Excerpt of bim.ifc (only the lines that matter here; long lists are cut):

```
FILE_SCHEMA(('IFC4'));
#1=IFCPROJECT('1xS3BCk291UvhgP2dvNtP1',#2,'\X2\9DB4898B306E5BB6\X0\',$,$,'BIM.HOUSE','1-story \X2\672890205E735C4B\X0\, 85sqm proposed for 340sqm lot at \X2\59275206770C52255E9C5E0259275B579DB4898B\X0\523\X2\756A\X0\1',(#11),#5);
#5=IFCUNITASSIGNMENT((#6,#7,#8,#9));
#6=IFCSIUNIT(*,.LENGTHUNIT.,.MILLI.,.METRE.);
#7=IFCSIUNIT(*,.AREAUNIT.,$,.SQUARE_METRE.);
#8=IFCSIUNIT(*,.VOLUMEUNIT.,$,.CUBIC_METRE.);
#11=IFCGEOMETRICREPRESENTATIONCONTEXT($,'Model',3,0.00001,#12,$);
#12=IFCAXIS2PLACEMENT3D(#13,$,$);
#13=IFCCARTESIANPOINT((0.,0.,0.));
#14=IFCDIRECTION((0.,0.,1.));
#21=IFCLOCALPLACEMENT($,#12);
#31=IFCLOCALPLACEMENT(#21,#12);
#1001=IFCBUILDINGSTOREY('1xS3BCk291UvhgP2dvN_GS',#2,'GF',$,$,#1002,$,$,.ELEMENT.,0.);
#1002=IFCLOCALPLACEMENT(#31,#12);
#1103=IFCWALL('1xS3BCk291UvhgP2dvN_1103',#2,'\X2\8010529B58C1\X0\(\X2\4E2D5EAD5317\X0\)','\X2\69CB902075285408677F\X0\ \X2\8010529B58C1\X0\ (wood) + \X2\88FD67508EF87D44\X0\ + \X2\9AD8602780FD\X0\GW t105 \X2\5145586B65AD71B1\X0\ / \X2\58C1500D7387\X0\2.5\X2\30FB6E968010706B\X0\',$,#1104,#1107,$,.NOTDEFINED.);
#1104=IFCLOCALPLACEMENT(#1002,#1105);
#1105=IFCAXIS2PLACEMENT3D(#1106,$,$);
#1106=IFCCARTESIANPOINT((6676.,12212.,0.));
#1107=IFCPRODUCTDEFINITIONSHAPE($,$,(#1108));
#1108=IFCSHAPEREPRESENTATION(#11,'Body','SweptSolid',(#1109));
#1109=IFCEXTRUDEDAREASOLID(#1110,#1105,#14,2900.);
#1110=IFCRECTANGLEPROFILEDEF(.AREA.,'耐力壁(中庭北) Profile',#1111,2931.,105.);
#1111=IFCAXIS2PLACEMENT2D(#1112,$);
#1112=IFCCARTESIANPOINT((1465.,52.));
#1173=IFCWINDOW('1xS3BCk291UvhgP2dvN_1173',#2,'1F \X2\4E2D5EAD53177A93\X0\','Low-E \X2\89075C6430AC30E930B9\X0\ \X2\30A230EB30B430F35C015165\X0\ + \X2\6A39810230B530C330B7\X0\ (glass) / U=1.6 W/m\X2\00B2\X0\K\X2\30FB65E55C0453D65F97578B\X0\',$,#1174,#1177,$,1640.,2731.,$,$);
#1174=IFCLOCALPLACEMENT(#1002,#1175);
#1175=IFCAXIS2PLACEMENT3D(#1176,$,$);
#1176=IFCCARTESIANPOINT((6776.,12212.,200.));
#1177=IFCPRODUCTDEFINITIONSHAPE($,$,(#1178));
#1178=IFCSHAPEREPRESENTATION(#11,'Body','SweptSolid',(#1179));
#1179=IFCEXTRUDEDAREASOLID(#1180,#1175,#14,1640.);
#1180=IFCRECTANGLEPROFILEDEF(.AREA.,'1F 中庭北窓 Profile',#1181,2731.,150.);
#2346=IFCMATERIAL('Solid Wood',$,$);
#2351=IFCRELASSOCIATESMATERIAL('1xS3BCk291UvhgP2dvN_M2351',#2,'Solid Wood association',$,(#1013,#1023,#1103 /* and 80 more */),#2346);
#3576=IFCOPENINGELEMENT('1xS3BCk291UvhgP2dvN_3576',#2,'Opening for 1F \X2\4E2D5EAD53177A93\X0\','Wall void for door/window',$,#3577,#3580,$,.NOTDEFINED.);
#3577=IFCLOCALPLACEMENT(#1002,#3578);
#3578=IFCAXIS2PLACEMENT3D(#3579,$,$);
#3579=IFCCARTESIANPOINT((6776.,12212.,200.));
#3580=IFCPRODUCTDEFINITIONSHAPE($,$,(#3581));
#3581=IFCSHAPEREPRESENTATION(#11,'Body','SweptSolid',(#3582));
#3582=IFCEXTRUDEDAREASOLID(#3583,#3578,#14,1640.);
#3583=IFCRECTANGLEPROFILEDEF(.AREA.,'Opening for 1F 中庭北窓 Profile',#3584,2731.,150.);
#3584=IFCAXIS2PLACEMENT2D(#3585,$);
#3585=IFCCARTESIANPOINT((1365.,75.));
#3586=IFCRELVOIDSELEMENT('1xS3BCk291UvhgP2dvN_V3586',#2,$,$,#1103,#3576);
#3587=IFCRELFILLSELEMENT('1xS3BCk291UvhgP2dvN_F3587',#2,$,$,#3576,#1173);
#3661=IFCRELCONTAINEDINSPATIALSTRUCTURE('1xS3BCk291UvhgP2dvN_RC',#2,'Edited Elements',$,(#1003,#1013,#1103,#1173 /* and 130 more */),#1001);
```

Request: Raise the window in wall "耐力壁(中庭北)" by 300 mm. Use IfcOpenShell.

```python
import numpy as np
import ifcopenshell
import ifcopenshell.api.geometry
import ifcopenshell.util.placement
import ifcopenshell.util.unit

model = ifcopenshell.open("bim.ifc")
unit_scale = ifcopenshell.util.unit.calculate_unit_scale(model)

window = model.by_guid("1xS3BCk291UvhgP2dvN_1173")
opening = window.FillsVoids[0].RelatingOpeningElement
dz = 0.3 / unit_scale

shift = np.array([0.0, 0.0, dz])
# The window is not placed relative to its opening, so move both.
for product in (opening, window):
    matrix = ifcopenshell.util.placement.get_local_placement(product.ObjectPlacement)
    matrix[:3, 3] += shift
    ifcopenshell.api.geometry.edit_object_placement(model, product=product, matrix=matrix, is_si=False)

print(f"moved by {dz * unit_scale:+.3f} m")

model.write("bim_edited.ifc")
```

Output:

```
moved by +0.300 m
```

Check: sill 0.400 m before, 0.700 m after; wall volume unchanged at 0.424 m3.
